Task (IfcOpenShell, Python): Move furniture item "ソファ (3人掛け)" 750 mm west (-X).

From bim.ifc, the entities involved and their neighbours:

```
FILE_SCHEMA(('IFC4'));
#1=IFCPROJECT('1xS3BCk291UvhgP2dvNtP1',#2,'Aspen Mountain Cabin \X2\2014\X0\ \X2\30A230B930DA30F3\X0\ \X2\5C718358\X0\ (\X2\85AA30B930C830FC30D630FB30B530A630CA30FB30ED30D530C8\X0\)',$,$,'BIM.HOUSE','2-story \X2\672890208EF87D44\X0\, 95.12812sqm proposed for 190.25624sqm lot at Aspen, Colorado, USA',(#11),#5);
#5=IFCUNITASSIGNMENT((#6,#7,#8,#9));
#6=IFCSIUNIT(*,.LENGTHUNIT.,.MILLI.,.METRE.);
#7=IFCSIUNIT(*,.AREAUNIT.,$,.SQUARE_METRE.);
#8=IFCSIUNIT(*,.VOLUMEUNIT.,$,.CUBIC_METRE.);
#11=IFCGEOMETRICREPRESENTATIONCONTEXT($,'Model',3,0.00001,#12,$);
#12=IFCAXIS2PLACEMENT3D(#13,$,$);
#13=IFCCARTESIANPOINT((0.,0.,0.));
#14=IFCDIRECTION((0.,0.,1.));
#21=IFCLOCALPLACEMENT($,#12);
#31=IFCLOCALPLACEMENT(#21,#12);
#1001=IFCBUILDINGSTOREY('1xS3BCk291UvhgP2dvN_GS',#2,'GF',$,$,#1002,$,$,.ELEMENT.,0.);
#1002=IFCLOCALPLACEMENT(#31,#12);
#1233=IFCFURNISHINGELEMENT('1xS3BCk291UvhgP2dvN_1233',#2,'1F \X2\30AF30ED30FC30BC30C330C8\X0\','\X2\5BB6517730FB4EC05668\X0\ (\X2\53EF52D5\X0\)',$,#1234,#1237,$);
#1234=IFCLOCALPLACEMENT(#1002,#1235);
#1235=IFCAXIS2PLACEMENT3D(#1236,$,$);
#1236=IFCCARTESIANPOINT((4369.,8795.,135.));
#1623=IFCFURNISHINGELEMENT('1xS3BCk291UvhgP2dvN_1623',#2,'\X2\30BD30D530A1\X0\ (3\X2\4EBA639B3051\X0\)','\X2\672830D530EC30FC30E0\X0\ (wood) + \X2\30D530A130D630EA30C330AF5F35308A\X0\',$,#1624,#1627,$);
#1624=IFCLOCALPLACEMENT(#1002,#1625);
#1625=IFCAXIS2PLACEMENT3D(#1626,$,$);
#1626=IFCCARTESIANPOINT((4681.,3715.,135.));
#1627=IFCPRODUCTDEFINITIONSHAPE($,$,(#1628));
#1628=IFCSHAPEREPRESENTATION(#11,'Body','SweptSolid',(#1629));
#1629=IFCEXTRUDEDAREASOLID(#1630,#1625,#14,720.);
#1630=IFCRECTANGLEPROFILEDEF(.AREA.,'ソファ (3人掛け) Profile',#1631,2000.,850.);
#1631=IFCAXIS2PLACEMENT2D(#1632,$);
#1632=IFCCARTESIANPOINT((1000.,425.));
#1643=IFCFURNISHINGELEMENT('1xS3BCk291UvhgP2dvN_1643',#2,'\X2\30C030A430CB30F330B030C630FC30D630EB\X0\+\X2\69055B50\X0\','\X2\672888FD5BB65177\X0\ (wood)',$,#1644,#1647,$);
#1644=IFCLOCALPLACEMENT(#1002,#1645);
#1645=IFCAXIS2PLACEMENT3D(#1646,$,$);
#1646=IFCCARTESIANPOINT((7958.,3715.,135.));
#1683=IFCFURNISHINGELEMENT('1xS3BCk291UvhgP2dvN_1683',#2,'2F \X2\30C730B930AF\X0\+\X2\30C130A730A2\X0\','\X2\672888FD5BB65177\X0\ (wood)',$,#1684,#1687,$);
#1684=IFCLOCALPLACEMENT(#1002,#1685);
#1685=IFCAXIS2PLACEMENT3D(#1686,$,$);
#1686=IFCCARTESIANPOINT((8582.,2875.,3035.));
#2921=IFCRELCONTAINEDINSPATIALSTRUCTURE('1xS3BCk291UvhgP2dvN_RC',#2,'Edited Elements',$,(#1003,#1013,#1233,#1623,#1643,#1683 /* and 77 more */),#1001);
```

```python
import ifcopenshell
import ifcopenshell.api.geometry
import ifcopenshell.util.placement
import ifcopenshell.util.unit

model = ifcopenshell.open("bim.ifc")
unit_scale = ifcopenshell.util.unit.calculate_unit_scale(model)

item = model.by_guid("1xS3BCk291UvhgP2dvN_1623")
matrix = ifcopenshell.util.placement.get_local_placement(item.ObjectPlacement)
matrix[0, 3] -= 0.75 / unit_scale
ifcopenshell.api.geometry.edit_object_placement(model, product=item, matrix=matrix, is_si=False)

print(ifcopenshell.util.placement.get_local_placement(item.ObjectPlacement).round(3) + 0.0)

model.write("bim_v2.ifc")
```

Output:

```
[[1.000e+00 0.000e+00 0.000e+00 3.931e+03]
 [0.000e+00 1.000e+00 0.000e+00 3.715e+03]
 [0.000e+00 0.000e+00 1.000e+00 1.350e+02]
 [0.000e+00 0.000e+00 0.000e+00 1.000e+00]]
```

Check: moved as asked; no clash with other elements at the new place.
